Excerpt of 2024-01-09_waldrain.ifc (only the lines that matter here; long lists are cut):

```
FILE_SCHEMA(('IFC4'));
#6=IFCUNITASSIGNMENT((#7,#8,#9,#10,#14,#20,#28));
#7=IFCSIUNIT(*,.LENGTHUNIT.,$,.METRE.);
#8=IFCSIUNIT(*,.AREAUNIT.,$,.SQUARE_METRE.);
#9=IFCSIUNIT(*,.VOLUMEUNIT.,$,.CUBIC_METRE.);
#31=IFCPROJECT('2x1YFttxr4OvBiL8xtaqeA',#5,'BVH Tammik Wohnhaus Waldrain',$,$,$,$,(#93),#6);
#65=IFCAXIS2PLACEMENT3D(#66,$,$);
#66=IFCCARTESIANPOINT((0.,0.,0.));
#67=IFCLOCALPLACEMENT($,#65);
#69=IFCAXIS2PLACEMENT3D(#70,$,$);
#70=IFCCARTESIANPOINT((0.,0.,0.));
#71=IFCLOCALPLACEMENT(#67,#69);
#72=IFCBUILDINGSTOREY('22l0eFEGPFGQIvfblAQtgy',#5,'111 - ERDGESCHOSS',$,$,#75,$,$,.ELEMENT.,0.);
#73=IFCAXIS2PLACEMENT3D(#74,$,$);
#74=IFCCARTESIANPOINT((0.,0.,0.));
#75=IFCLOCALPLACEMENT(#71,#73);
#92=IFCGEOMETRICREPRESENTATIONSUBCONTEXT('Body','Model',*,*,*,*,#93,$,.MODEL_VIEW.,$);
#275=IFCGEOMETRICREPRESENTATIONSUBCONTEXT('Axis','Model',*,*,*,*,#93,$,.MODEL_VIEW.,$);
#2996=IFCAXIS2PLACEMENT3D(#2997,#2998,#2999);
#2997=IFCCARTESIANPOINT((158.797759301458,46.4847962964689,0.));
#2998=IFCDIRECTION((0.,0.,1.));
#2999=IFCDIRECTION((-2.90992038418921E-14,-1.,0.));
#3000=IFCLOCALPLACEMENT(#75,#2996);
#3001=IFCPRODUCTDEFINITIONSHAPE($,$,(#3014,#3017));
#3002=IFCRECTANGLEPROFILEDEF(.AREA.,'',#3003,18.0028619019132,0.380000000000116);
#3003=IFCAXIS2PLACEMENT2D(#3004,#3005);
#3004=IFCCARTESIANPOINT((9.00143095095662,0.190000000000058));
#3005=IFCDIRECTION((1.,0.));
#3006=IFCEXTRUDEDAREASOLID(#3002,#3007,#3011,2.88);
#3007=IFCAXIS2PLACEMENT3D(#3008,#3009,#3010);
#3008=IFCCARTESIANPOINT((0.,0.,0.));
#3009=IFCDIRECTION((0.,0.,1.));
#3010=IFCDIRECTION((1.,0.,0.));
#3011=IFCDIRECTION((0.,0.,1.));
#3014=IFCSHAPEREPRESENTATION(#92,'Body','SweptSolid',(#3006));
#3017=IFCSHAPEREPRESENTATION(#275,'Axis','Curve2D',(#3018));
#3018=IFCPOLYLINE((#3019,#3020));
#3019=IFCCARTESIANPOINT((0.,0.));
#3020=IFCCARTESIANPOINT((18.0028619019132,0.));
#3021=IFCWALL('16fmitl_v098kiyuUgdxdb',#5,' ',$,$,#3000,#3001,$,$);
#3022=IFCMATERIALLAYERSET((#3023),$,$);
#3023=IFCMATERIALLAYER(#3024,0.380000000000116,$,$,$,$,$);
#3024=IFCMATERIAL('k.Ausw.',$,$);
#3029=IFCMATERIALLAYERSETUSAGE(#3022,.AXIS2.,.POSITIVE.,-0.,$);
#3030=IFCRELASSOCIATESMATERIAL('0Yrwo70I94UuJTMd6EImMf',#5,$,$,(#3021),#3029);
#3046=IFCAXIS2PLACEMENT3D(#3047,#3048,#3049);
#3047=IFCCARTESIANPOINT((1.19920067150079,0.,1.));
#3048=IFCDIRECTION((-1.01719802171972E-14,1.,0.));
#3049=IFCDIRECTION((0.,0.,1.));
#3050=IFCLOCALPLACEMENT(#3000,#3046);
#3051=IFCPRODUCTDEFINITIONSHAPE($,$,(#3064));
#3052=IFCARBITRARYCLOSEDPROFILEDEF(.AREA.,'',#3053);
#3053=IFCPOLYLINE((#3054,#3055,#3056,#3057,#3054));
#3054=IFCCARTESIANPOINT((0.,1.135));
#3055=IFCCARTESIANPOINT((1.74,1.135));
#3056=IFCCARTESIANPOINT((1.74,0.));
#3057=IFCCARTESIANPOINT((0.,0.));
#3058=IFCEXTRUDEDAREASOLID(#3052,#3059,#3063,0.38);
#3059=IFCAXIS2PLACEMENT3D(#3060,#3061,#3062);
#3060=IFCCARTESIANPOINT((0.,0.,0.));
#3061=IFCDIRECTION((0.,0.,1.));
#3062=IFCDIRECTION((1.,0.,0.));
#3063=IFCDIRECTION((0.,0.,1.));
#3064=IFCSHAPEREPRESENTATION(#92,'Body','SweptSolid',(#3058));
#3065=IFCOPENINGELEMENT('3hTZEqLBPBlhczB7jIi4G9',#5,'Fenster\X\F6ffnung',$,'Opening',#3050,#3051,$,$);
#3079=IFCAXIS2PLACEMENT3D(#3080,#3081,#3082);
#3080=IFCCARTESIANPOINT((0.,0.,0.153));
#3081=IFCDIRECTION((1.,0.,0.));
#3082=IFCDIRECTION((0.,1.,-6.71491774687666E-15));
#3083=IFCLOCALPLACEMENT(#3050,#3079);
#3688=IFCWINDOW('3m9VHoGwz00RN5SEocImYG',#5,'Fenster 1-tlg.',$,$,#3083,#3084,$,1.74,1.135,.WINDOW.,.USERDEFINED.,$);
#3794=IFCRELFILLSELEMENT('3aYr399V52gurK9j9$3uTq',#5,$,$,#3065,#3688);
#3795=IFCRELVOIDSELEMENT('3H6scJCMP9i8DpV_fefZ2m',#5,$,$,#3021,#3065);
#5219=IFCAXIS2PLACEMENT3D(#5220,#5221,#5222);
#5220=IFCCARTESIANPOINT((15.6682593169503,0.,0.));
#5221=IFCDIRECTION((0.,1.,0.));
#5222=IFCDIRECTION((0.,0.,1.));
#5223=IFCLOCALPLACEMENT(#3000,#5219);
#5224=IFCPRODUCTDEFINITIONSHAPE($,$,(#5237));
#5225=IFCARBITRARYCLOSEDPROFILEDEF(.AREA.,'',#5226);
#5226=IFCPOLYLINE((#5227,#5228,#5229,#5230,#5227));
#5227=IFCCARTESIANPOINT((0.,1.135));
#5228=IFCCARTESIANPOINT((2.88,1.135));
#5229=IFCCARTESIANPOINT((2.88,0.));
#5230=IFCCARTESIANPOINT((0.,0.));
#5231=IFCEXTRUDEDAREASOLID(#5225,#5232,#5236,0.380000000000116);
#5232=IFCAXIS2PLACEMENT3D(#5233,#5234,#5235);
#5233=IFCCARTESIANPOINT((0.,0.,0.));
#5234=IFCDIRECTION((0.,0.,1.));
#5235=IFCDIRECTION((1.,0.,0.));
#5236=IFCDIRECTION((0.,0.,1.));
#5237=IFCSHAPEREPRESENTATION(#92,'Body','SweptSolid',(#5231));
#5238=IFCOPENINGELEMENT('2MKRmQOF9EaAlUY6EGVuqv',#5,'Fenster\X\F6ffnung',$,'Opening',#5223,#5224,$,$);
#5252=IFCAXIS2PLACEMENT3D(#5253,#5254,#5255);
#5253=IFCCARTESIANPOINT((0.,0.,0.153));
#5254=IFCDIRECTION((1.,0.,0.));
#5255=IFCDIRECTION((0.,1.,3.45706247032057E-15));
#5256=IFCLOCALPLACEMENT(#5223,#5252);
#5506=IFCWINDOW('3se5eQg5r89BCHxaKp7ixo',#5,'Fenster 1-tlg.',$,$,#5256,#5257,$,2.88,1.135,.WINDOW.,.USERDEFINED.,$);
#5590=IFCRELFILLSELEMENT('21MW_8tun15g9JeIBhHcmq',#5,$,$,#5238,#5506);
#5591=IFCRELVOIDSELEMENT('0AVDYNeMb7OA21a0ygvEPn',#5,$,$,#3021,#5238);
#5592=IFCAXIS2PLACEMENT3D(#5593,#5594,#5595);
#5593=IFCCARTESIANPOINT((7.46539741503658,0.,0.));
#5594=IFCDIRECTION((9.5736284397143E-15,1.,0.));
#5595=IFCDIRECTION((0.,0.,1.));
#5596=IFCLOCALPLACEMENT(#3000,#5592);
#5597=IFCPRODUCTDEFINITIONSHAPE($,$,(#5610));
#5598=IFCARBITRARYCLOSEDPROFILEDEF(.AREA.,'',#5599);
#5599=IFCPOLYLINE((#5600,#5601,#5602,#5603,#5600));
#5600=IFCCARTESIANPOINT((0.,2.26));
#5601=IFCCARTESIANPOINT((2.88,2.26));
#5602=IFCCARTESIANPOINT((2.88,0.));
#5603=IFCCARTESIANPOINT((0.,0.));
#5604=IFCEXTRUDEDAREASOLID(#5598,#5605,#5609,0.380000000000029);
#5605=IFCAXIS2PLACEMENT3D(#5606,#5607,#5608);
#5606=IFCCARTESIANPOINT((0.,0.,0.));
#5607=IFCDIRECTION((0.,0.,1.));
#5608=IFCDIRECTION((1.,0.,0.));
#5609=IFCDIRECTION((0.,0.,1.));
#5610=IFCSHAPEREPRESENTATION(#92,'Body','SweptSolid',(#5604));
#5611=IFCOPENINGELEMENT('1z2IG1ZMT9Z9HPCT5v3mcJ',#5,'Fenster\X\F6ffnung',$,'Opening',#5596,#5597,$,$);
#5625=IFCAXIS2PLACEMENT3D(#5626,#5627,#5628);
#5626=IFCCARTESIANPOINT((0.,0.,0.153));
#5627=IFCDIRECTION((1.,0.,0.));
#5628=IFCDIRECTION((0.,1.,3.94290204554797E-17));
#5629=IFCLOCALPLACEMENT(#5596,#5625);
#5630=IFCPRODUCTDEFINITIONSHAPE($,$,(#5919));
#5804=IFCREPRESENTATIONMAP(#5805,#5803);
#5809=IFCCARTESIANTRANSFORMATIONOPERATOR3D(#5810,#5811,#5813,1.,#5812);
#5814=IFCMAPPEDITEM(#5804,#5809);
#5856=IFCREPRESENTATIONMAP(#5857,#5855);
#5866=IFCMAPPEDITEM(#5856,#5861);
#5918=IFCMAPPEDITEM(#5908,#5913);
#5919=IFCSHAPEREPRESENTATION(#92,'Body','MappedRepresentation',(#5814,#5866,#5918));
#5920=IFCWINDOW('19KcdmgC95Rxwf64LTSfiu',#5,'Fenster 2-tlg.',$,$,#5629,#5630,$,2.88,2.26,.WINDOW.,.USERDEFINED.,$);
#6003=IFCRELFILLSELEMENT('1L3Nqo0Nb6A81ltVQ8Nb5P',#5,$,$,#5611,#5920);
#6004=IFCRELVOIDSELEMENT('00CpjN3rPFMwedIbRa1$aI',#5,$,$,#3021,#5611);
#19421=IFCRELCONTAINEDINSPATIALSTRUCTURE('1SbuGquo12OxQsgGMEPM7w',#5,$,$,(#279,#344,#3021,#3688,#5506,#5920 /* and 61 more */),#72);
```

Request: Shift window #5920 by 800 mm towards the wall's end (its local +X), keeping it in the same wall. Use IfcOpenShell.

```python
import ifcopenshell
import ifcopenshell.api.geometry
import ifcopenshell.util.placement
import ifcopenshell.util.unit

model = ifcopenshell.open("2024-01-09_waldrain.ifc")
unit_scale = ifcopenshell.util.unit.calculate_unit_scale(model)

window = model.by_id(5920)
opening = window.FillsVoids[0].RelatingOpeningElement
wall = opening.VoidsElements[0].RelatingBuildingElement

wall_matrix = ifcopenshell.util.placement.get_local_placement(wall.ObjectPlacement)
shift = wall_matrix[:3, 0] * 0.8 / unit_scale
before = ifcopenshell.util.placement.get_local_placement(window.ObjectPlacement)[:3, 3].copy()

# The window is placed relative to its opening, so it follows when the opening moves.
matrix = ifcopenshell.util.placement.get_local_placement(opening.ObjectPlacement)
matrix[:3, 3] += shift
ifcopenshell.api.geometry.edit_object_placement(
    model, product=opening, matrix=matrix, is_si=False, should_transform_children=True
)

after = ifcopenshell.util.placement.get_local_placement(window.ObjectPlacement)[:3, 3]
print("window moved by", (after - before).round(3) + 0.0)

model.write("2024-01-09_waldrain_updated.ifc")
```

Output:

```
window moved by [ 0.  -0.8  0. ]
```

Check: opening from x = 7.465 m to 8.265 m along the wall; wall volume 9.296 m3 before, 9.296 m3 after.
